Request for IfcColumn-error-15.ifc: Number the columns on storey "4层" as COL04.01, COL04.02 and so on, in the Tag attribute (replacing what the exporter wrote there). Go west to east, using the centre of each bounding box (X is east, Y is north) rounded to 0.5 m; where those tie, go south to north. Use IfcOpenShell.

First a look at what the model holds.

```python
import ifcopenshell
import ifcopenshell.util.element
import ifcopenshell.util.placement

model = ifcopenshell.open("IfcColumn-error-15.ifc")
print(model.schema)
storey = next(s for s in model.by_type("IfcBuildingStorey") if s.Name == "4层")
columns = [e for e in ifcopenshell.util.element.get_decomposition(storey) if e.is_a("IfcColumn")]
for e in sorted(columns, key=lambda e: e.id()):
    origin = ifcopenshell.util.placement.get_local_placement(e.ObjectPlacement)[:3, 3]
    print(e.id(), e.Tag, e.Name, origin.round(2) + 0.0, sep=" | ")
```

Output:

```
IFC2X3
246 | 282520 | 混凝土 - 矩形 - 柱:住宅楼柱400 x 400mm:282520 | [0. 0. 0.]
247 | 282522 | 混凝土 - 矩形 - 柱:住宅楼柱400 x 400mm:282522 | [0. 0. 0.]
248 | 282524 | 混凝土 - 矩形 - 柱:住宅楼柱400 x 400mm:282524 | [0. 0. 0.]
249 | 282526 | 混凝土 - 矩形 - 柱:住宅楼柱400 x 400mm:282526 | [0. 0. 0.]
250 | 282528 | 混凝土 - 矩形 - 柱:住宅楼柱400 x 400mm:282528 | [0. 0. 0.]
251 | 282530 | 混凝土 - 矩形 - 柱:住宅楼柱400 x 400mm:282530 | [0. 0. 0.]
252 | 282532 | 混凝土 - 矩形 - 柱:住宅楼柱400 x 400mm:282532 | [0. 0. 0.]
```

```python
import ifcopenshell
import ifcopenshell.geom
import ifcopenshell.util.element
import ifcopenshell.util.shape

model = ifcopenshell.open("IfcColumn-error-15.ifc")
settings = ifcopenshell.geom.settings()
settings.set("use-world-coords", True)


def centre(element):
    shape = ifcopenshell.geom.create_shape(settings, element)
    return ifcopenshell.util.shape.get_bbox_centroid(shape.geometry)


storey = next(s for s in model.by_type("IfcBuildingStorey") if s.Name == "4层")
columns = [e for e in ifcopenshell.util.element.get_decomposition(storey) if e.is_a("IfcColumn")]

# Insertion points can sit at a corner or the storey origin, so sort by the geometry (in metres).
centres = {e: centre(e) for e in columns}
columns.sort(key=lambda e: (round(centres[e][0] / 0.5), centres[e][1]))

for i, e in enumerate(columns, start=1):
    number = f"COL04.{i:02d}"
    e.Tag = number
    print(e.id(), number)

model.write("IfcColumn-error-15_v2.ifc")
```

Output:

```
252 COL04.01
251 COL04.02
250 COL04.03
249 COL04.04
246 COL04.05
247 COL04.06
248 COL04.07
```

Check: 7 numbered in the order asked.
